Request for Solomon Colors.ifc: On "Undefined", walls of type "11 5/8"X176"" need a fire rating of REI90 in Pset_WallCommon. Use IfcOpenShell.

First a look at what the model holds.

```python
import ifcopenshell
import ifcopenshell.util.element

model = ifcopenshell.open("Solomon Colors.ifc")
print(model.schema)
storey = next(s for s in model.by_type("IfcBuildingStorey") if s.Name == "Undefined")
walls = [e for e in ifcopenshell.util.element.get_decomposition(storey) if e.is_a("IfcWall")]
seen = {}
for e in walls:
    element_type = ifcopenshell.util.element.get_type(e)
    key = (element_type.Name if element_type != e and element_type else None, ifcopenshell.util.element.get_pset(e, "Pset_WallCommon", "FireRating"))
    seen[key] = seen.get(key, 0) + 1
for (name, value), count in sorted(seen.items(), key=str):
    print(count, "x", name, "|", value)
```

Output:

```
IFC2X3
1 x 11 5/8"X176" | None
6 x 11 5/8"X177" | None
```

```python
import ifcopenshell
import ifcopenshell.api.pset
import ifcopenshell.util.element

model = ifcopenshell.open("Solomon Colors.ifc")

storey = next(s for s in model.by_type("IfcBuildingStorey") if s.Name == "Undefined")
walls = [e for e in ifcopenshell.util.element.get_decomposition(storey) if e.is_a("IfcWall")]

count = 0
for e in walls:
    element_type = ifcopenshell.util.element.get_type(e)
    if element_type in (None, e) or element_type.Name != '11 5/8"X176"':
        continue
    # add_pset returns the element's existing set when there is one.
    pset = ifcopenshell.api.pset.add_pset(model, product=e, name="Pset_WallCommon")
    ifcopenshell.api.pset.edit_pset(model, pset=pset, properties={"FireRating": "REI90"})
    count += 1

print(count, "walls updated")

model.write("Solomon Colors_v2.ifc")
```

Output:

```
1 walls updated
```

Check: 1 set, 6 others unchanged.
